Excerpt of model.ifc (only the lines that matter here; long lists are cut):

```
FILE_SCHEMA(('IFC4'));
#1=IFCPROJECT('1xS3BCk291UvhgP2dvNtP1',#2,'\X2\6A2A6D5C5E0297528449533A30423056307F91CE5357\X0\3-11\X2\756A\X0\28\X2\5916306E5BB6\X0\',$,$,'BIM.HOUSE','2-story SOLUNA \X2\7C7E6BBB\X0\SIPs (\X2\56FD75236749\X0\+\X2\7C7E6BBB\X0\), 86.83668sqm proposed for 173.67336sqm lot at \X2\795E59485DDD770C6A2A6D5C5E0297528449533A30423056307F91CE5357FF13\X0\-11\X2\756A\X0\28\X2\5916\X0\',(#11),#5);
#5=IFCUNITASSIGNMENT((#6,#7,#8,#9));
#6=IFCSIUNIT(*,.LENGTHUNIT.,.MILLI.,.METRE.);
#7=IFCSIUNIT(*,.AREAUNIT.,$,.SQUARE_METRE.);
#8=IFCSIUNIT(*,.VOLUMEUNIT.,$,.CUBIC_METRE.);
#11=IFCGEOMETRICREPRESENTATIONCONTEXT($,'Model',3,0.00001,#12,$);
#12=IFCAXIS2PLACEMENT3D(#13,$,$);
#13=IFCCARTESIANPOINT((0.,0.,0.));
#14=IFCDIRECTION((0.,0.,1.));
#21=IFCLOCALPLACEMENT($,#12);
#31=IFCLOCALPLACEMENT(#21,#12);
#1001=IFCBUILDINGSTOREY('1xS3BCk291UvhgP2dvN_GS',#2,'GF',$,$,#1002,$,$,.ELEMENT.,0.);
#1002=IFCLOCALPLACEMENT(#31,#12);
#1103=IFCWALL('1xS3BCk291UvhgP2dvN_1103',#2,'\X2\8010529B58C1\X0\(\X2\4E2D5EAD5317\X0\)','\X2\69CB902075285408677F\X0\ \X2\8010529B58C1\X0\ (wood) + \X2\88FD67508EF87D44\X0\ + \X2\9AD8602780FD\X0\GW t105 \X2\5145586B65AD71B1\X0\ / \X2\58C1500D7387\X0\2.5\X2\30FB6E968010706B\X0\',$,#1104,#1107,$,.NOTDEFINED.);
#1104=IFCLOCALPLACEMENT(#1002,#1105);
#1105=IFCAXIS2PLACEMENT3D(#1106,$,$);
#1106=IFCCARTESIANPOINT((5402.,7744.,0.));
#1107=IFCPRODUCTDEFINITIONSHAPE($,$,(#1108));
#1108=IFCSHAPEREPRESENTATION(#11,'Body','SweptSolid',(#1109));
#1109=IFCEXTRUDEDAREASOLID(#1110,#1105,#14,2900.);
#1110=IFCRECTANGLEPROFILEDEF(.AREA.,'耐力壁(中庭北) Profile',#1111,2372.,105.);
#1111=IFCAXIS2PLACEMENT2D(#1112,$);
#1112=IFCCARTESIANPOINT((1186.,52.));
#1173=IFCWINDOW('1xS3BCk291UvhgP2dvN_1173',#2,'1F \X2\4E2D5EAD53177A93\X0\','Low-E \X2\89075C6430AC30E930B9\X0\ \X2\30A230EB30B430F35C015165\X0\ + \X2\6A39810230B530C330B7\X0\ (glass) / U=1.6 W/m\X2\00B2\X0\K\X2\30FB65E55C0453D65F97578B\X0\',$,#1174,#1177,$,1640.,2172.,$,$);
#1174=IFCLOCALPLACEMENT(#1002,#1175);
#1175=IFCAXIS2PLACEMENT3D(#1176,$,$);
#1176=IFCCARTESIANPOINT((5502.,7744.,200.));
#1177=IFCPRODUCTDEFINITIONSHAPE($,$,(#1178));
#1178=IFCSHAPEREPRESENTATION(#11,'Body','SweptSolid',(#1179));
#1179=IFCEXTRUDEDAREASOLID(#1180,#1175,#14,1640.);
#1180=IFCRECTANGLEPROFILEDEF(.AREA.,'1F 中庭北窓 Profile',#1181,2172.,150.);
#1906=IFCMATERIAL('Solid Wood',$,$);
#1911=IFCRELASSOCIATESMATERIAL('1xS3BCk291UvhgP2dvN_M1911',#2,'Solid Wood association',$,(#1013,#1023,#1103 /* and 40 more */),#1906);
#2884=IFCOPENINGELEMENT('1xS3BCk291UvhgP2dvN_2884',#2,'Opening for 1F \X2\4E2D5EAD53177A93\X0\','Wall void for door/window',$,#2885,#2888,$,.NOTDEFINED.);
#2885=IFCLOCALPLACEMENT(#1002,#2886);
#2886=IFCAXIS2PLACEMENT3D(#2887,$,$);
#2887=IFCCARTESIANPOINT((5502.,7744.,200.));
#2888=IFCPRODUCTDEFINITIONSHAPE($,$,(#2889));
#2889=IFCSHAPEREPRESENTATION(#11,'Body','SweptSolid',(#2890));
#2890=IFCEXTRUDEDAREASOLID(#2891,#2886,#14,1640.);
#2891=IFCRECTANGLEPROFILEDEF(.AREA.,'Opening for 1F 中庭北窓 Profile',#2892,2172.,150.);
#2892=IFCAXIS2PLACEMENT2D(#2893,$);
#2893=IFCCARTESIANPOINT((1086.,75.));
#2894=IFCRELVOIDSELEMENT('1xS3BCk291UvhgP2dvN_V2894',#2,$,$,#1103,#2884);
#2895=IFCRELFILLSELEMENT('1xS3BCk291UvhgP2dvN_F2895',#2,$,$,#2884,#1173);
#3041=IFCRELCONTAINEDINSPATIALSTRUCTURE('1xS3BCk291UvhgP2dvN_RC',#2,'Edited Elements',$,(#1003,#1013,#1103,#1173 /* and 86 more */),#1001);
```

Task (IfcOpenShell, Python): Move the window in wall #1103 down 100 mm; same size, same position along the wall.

```python
import numpy as np
import ifcopenshell
import ifcopenshell.api.geometry
import ifcopenshell.util.placement
import ifcopenshell.util.unit

model = ifcopenshell.open("model.ifc")
unit_scale = ifcopenshell.util.unit.calculate_unit_scale(model)

window = model.by_id(1173)
opening = window.FillsVoids[0].RelatingOpeningElement
dz = -0.1 / unit_scale

shift = np.array([0.0, 0.0, dz])
# The window is not placed relative to its opening, so move both.
for product in (opening, window):
    matrix = ifcopenshell.util.placement.get_local_placement(product.ObjectPlacement)
    matrix[:3, 3] += shift
    ifcopenshell.api.geometry.edit_object_placement(model, product=product, matrix=matrix, is_si=False)

print(f"moved by {dz * unit_scale:+.3f} m")

model.write("model-out.ifc")
```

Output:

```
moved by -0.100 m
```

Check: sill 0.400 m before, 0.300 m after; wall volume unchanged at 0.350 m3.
